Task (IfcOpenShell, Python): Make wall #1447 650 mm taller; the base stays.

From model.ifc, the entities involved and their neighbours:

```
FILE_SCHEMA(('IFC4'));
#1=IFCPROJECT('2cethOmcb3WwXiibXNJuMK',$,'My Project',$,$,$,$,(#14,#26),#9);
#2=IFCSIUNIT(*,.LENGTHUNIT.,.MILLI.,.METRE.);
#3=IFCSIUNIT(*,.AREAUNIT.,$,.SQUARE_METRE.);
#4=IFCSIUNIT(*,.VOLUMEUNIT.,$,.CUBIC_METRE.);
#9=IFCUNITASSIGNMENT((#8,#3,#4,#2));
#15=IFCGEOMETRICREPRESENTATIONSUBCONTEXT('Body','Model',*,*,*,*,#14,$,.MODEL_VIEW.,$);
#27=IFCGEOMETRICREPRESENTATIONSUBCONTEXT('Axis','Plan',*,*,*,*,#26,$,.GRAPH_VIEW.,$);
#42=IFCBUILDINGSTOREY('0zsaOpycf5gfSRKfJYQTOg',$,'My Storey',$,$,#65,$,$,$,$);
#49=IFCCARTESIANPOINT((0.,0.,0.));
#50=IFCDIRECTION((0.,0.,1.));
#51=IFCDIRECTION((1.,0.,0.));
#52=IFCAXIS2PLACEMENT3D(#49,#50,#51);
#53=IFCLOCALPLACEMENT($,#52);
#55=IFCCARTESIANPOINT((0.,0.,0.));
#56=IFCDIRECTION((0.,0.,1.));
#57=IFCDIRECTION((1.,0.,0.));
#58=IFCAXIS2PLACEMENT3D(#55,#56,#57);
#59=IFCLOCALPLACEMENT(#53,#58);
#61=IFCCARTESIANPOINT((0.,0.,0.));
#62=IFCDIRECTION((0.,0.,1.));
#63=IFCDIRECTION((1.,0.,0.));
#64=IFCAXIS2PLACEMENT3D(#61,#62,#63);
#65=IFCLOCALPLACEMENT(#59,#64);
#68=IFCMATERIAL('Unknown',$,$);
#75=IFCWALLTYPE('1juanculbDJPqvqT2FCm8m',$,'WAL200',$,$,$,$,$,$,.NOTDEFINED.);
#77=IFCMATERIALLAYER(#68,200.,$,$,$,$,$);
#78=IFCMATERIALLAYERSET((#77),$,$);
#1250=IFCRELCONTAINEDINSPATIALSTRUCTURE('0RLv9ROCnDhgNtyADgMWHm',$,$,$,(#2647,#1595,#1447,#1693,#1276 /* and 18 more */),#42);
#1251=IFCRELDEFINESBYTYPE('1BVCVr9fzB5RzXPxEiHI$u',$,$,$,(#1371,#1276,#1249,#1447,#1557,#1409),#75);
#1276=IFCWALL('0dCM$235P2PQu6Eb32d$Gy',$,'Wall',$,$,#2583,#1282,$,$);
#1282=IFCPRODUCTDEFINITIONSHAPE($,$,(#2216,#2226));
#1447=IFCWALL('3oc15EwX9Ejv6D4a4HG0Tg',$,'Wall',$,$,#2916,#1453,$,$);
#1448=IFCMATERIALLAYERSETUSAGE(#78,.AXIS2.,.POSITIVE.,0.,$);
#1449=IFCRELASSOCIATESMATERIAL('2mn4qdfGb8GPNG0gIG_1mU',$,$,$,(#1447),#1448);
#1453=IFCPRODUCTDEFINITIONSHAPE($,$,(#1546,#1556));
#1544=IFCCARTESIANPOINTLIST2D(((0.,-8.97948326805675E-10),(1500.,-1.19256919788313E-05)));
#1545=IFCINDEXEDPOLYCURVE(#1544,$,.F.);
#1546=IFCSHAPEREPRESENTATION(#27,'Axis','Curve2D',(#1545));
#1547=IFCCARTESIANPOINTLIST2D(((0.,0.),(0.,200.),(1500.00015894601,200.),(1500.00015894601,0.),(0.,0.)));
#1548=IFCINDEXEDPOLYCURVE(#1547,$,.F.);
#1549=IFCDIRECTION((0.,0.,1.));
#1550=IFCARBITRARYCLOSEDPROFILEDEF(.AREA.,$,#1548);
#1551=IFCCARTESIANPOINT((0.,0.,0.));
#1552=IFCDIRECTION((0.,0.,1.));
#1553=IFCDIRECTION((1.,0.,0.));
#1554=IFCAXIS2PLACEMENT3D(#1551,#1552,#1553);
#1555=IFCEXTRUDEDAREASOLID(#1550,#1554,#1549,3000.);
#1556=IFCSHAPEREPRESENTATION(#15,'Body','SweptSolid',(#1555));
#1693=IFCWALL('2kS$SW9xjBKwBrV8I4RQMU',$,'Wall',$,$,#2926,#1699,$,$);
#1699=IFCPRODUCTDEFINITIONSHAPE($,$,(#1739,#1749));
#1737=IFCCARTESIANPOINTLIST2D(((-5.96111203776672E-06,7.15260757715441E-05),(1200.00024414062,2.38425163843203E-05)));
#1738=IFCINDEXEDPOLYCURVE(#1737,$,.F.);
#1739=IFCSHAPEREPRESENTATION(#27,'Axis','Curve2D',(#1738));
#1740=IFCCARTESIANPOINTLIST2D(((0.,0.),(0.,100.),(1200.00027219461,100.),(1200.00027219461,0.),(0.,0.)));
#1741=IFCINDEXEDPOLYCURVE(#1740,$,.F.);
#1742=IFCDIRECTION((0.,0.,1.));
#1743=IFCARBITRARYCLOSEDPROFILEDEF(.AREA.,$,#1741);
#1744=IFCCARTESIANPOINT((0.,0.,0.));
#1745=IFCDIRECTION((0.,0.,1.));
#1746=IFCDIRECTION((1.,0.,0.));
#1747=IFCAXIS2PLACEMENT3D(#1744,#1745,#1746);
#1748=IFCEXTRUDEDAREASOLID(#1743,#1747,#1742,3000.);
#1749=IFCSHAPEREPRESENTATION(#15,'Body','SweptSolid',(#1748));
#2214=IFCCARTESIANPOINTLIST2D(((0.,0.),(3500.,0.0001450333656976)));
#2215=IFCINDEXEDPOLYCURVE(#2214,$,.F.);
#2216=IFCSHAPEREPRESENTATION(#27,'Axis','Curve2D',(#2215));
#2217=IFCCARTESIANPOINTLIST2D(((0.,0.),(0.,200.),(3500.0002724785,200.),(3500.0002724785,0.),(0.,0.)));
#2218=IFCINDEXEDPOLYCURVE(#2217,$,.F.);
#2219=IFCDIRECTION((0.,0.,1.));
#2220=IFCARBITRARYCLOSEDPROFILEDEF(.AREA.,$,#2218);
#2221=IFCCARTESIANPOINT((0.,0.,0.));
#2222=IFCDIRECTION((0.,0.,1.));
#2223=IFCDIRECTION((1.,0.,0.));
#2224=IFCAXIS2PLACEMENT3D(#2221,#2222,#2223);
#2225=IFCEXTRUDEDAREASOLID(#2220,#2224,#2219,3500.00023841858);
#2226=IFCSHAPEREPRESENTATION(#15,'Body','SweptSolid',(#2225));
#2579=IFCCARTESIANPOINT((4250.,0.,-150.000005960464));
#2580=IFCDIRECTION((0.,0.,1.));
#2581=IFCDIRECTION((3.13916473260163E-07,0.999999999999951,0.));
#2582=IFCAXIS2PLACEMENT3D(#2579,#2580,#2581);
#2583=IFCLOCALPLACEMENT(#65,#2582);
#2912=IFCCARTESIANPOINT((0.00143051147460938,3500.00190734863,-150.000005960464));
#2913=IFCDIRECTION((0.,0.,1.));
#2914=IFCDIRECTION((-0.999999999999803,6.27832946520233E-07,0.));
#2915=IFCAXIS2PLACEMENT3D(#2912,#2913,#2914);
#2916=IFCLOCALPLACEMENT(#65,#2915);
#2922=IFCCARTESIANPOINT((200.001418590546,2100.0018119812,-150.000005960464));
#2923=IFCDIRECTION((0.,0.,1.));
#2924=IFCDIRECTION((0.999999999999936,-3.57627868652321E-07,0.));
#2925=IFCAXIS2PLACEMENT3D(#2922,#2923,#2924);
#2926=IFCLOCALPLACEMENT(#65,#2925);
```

```python
import ifcopenshell
import ifcopenshell.geom
import ifcopenshell.util.representation
import ifcopenshell.util.shape
import ifcopenshell.util.unit

model = ifcopenshell.open("model.ifc")
unit_scale = ifcopenshell.util.unit.calculate_unit_scale(model)
settings = ifcopenshell.geom.settings()


def volume(element):
    """Net volume in cubic metres, openings subtracted."""
    shape = ifcopenshell.geom.create_shape(settings, element)
    return ifcopenshell.util.shape.get_volume(shape.geometry)


wall = model.by_id(1447)
before = volume(wall)

body = ifcopenshell.util.representation.get_representation(wall, "Model", "Body")
solid = body.Items[0]
old_height = solid.Depth
solid.Depth += 0.65 / unit_scale
after = volume(wall)

print(f"height {old_height:g} -> {solid.Depth:g}, volume {before:.3f} -> {after:.3f} m3")

model.write("model_rev.ifc")
```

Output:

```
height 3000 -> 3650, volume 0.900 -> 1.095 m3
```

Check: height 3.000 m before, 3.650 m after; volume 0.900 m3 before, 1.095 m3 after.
